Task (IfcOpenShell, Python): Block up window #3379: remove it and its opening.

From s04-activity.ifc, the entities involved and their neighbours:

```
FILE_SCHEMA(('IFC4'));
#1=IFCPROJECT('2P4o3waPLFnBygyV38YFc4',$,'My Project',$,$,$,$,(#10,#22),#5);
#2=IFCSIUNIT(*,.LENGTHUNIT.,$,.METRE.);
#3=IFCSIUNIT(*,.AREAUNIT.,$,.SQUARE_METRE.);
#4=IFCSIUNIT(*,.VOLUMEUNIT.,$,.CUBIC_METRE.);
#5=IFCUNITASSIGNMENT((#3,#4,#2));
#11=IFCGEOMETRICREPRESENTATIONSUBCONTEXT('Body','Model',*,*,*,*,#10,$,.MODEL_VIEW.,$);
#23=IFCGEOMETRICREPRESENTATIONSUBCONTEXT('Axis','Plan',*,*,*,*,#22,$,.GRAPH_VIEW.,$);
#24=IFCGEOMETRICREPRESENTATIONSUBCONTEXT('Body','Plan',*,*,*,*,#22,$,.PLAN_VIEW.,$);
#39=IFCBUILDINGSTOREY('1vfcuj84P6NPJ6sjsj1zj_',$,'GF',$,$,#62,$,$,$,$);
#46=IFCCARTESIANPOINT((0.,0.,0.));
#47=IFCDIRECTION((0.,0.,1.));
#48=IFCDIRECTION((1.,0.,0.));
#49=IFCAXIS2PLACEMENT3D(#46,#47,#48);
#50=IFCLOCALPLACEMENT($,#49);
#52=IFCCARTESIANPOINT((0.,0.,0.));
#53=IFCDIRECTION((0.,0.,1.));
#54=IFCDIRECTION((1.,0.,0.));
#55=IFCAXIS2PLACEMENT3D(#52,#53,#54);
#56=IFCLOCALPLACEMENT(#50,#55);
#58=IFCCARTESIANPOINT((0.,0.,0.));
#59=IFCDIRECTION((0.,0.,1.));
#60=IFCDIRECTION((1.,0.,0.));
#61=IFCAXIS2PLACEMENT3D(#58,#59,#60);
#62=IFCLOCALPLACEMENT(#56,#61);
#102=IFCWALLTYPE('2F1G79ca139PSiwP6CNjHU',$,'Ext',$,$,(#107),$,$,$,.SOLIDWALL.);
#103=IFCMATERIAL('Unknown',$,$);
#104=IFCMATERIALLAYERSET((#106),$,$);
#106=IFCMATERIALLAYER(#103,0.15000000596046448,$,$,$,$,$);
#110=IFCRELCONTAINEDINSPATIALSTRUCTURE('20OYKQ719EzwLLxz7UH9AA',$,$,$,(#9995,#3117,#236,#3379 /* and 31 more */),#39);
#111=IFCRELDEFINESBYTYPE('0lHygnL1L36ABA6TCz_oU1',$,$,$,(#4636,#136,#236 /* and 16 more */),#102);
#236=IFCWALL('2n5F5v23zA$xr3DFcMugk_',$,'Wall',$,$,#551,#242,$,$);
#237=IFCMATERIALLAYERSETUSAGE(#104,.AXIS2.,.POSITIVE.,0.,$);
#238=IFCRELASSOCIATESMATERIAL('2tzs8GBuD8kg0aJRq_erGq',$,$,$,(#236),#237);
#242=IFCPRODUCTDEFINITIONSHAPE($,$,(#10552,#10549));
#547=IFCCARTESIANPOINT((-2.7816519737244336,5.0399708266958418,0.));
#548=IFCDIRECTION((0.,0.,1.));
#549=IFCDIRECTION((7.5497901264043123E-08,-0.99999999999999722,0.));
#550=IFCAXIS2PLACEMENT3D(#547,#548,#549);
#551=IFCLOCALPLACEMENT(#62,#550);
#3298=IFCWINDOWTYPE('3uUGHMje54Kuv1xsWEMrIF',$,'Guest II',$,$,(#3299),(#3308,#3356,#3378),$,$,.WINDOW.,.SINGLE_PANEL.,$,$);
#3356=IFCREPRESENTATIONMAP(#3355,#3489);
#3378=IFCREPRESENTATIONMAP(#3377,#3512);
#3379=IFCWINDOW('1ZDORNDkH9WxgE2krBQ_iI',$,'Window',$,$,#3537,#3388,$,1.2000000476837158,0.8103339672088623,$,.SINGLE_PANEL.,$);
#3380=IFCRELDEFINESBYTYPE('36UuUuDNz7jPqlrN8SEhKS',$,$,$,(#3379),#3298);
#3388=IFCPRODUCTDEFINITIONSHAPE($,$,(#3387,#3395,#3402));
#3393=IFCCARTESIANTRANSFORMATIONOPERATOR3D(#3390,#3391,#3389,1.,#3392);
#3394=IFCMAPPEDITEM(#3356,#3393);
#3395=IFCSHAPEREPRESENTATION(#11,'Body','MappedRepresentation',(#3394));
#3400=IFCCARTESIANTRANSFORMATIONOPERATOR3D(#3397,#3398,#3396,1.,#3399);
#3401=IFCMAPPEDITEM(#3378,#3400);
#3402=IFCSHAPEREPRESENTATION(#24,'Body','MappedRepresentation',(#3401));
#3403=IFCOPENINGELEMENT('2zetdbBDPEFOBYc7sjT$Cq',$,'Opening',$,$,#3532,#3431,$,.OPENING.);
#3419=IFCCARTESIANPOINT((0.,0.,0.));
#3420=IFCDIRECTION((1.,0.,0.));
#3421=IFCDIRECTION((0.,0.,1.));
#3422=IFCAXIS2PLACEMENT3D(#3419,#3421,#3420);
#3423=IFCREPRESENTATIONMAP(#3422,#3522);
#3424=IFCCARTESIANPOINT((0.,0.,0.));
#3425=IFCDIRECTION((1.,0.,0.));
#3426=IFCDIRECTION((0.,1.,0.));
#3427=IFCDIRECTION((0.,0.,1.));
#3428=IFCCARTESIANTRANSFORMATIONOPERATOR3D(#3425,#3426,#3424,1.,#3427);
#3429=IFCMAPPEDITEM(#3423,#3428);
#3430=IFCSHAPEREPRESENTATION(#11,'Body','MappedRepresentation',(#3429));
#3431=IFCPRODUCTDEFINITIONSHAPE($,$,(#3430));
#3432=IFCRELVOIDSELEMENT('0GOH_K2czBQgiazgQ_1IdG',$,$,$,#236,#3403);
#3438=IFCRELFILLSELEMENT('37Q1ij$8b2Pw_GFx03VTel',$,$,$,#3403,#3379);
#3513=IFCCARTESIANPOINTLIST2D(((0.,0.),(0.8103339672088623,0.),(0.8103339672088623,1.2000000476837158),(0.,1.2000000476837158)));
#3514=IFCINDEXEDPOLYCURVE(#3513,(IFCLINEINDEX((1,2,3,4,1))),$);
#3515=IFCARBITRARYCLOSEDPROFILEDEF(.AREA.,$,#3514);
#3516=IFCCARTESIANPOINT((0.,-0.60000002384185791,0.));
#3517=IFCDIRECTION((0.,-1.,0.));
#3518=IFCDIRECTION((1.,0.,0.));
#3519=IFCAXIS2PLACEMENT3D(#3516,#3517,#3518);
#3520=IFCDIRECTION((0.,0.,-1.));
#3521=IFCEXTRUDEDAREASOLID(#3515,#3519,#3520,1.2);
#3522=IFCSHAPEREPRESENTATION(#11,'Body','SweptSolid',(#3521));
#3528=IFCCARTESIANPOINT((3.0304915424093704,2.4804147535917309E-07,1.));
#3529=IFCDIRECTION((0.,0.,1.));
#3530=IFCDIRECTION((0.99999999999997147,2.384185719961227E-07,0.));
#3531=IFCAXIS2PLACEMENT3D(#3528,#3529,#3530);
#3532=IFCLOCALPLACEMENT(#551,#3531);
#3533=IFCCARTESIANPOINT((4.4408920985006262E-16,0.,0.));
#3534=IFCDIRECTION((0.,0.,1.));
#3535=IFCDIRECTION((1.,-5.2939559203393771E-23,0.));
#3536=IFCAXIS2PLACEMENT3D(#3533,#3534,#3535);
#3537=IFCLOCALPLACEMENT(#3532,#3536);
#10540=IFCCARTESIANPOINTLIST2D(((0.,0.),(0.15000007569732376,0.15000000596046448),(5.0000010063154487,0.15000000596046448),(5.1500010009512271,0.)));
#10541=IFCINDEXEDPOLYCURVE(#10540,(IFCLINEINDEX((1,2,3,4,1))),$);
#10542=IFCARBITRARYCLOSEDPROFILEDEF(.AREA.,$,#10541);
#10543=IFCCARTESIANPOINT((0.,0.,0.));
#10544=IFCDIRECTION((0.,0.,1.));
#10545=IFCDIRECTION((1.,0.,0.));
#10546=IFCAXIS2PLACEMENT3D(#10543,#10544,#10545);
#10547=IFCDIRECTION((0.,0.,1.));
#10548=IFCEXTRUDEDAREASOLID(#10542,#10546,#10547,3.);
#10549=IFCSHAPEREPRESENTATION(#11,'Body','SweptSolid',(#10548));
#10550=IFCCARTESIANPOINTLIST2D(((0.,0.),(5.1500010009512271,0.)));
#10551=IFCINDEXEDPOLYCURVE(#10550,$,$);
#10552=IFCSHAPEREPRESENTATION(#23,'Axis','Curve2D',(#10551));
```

```python
import ifcopenshell
import ifcopenshell.api.feature
import ifcopenshell.api.root
import ifcopenshell.geom
import ifcopenshell.util.shape

model = ifcopenshell.open("s04-activity.ifc")
settings = ifcopenshell.geom.settings()


def volume(element):
    """Net volume in cubic metres, openings subtracted."""
    shape = ifcopenshell.geom.create_shape(settings, element)
    return ifcopenshell.util.shape.get_volume(shape.geometry)


window = model.by_id(3379)
opening = window.FillsVoids[0].RelatingOpeningElement
wall = opening.VoidsElements[0].RelatingBuildingElement
before = volume(wall)

ifcopenshell.api.root.remove_product(model, product=window)
ifcopenshell.api.feature.remove_feature(model, feature=opening)

after = volume(wall)

print(f"wall volume {before:.3f} -> {after:.3f} m3")

model.write("s04-activity-out.ifc")
```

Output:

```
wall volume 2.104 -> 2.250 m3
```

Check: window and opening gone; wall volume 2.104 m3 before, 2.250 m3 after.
